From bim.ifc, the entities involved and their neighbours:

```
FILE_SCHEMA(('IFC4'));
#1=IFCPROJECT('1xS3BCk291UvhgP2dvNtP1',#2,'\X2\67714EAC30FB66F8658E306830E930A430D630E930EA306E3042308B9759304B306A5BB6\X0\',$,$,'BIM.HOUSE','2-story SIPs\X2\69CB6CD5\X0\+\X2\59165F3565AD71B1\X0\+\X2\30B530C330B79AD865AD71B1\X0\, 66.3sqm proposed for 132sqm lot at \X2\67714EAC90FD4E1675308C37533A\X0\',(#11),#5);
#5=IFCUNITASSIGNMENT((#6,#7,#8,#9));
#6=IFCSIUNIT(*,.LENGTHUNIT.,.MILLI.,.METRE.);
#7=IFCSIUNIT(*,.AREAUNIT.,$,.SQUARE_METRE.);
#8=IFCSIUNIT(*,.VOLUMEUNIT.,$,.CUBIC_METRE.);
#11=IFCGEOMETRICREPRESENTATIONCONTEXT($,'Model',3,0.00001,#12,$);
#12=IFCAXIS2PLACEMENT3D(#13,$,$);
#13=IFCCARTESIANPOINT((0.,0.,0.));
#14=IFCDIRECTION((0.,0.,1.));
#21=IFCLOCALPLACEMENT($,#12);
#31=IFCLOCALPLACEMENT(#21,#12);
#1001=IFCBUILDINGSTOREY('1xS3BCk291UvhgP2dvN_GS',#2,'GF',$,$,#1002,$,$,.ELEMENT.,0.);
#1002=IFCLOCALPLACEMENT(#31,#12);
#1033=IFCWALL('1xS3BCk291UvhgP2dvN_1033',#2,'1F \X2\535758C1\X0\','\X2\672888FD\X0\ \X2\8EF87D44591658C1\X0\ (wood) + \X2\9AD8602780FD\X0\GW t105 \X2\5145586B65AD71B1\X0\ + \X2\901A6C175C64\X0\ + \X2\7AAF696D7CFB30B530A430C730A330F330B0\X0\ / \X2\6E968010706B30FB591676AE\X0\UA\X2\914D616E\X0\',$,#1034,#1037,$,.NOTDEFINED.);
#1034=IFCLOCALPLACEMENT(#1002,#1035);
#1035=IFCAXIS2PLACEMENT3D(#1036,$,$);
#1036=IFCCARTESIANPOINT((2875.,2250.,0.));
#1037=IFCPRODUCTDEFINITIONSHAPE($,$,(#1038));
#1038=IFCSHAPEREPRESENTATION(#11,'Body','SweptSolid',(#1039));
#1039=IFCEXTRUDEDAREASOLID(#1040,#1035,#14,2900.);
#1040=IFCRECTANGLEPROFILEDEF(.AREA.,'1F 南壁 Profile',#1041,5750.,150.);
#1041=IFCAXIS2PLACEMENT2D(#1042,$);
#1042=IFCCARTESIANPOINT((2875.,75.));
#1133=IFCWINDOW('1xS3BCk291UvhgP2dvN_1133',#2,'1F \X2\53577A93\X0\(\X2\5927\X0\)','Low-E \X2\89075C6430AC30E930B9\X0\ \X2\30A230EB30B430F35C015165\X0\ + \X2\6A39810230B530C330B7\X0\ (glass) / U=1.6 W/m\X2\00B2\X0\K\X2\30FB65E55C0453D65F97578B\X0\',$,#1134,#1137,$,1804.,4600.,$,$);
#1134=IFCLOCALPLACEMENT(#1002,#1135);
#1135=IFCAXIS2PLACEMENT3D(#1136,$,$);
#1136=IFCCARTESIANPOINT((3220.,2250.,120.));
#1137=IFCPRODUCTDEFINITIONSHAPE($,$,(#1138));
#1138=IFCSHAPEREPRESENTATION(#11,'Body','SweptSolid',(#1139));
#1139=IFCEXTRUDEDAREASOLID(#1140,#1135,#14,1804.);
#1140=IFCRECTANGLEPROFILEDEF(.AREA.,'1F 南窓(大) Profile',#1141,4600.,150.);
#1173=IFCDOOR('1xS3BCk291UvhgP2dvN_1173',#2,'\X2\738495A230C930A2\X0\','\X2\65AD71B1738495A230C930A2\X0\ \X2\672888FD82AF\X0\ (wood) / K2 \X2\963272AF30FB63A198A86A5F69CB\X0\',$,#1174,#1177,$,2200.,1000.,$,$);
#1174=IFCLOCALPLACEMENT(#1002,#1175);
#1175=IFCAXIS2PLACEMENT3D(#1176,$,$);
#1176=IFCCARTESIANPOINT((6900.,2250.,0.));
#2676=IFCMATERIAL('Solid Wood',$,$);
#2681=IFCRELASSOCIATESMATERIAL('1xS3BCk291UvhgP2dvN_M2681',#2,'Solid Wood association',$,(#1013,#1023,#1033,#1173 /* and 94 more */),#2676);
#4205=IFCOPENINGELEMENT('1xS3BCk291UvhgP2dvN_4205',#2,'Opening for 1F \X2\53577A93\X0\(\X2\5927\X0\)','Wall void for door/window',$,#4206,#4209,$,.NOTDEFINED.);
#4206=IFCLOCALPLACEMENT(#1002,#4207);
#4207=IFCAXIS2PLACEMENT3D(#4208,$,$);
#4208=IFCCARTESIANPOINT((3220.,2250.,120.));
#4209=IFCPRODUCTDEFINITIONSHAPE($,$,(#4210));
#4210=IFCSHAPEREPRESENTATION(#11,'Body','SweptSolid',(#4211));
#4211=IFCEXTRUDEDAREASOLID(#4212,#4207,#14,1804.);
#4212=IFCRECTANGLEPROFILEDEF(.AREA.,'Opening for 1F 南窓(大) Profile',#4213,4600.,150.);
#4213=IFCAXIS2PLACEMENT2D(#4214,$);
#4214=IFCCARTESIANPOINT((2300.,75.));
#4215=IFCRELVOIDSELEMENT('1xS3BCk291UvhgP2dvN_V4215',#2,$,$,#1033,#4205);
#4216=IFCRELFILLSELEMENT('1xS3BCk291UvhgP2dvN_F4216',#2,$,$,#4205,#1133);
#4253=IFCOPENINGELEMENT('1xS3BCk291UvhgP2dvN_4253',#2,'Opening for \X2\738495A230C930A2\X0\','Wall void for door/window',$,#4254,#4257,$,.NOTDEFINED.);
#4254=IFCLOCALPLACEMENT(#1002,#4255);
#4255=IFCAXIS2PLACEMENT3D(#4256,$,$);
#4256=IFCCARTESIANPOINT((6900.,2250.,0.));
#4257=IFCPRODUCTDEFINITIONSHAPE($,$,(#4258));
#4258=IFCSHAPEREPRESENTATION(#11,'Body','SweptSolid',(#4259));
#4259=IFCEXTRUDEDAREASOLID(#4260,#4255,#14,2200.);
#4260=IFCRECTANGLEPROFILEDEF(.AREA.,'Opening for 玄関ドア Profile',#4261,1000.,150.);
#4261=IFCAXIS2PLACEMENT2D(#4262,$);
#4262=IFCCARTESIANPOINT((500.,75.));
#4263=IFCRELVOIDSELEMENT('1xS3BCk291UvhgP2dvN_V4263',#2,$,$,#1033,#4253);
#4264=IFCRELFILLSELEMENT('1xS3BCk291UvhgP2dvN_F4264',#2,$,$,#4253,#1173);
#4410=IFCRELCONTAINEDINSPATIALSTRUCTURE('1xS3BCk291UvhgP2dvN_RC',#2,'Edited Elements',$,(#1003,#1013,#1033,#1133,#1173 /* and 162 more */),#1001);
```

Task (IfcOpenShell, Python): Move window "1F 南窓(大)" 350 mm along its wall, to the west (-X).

```python
import ifcopenshell
import ifcopenshell.api.geometry
import ifcopenshell.util.placement
import ifcopenshell.util.unit

model = ifcopenshell.open("bim.ifc")
unit_scale = ifcopenshell.util.unit.calculate_unit_scale(model)

window = model.by_id(1133)
opening = window.FillsVoids[0].RelatingOpeningElement
wall = opening.VoidsElements[0].RelatingBuildingElement

wall_matrix = ifcopenshell.util.placement.get_local_placement(wall.ObjectPlacement)
shift = wall_matrix[:3, 0] * -0.35 / unit_scale
before = ifcopenshell.util.placement.get_local_placement(window.ObjectPlacement)[:3, 3].copy()

# The window is not placed relative to its opening, so move both.
for product in (opening, window):
    matrix = ifcopenshell.util.placement.get_local_placement(product.ObjectPlacement)
    matrix[:3, 3] += shift
    ifcopenshell.api.geometry.edit_object_placement(model, product=product, matrix=matrix, is_si=False)

after = ifcopenshell.util.placement.get_local_placement(window.ObjectPlacement)[:3, 3]
print("window moved by", (after - before).round(3) + 0.0)

model.write("bim_rev.ifc")
```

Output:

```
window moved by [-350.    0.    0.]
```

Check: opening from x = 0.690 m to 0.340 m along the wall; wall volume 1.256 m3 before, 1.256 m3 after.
